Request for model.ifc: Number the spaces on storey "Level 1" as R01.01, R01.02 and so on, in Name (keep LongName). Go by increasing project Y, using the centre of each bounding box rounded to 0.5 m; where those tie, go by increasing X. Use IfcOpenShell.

First a look at what the model holds.

```python
import ifcopenshell
import ifcopenshell.util.element
import ifcopenshell.util.placement

model = ifcopenshell.open("model.ifc")
print(model.schema)
storey = next(s for s in model.by_type("IfcBuildingStorey") if s.Name == "Level 1")
spaces = [e for e in ifcopenshell.util.element.get_decomposition(storey) if e.is_a("IfcSpace")]
for e in sorted(spaces, key=lambda e: e.id()):
    origin = ifcopenshell.util.placement.get_local_placement(e.ObjectPlacement)[:3, 3]
    print(e.id(), e.Name, e.LongName, origin.round(2) + 0.0, sep=" | ")
```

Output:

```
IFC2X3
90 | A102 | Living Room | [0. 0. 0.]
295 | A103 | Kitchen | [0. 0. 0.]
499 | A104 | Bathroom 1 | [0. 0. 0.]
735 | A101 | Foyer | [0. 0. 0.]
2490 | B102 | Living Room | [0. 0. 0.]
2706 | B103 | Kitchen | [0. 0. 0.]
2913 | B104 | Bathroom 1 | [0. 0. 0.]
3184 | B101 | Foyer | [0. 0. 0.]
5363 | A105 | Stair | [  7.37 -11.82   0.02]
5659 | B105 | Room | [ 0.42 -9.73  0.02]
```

```python
import ifcopenshell
import ifcopenshell.geom
import ifcopenshell.util.element
import ifcopenshell.util.shape

model = ifcopenshell.open("model.ifc")
settings = ifcopenshell.geom.settings()
settings.set("use-world-coords", True)


def centre(element):
    shape = ifcopenshell.geom.create_shape(settings, element)
    return ifcopenshell.util.shape.get_bbox_centroid(shape.geometry)


storey = next(s for s in model.by_type("IfcBuildingStorey") if s.Name == "Level 1")
spaces = [e for e in ifcopenshell.util.element.get_decomposition(storey) if e.is_a("IfcSpace")]

# Insertion points can sit at a corner or the storey origin, so sort by the geometry (in metres).
centres = {e: centre(e) for e in spaces}
spaces.sort(key=lambda e: (round(centres[e][1] / 0.5), centres[e][0]))

for i, e in enumerate(spaces, start=1):
    number = f"R01.{i:02d}"
    e.Name = number
    print(e.id(), number)

model.write("model_updated.ifc")
```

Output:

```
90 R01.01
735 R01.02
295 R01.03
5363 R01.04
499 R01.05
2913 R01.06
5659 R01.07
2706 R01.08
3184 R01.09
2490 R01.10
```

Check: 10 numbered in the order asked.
